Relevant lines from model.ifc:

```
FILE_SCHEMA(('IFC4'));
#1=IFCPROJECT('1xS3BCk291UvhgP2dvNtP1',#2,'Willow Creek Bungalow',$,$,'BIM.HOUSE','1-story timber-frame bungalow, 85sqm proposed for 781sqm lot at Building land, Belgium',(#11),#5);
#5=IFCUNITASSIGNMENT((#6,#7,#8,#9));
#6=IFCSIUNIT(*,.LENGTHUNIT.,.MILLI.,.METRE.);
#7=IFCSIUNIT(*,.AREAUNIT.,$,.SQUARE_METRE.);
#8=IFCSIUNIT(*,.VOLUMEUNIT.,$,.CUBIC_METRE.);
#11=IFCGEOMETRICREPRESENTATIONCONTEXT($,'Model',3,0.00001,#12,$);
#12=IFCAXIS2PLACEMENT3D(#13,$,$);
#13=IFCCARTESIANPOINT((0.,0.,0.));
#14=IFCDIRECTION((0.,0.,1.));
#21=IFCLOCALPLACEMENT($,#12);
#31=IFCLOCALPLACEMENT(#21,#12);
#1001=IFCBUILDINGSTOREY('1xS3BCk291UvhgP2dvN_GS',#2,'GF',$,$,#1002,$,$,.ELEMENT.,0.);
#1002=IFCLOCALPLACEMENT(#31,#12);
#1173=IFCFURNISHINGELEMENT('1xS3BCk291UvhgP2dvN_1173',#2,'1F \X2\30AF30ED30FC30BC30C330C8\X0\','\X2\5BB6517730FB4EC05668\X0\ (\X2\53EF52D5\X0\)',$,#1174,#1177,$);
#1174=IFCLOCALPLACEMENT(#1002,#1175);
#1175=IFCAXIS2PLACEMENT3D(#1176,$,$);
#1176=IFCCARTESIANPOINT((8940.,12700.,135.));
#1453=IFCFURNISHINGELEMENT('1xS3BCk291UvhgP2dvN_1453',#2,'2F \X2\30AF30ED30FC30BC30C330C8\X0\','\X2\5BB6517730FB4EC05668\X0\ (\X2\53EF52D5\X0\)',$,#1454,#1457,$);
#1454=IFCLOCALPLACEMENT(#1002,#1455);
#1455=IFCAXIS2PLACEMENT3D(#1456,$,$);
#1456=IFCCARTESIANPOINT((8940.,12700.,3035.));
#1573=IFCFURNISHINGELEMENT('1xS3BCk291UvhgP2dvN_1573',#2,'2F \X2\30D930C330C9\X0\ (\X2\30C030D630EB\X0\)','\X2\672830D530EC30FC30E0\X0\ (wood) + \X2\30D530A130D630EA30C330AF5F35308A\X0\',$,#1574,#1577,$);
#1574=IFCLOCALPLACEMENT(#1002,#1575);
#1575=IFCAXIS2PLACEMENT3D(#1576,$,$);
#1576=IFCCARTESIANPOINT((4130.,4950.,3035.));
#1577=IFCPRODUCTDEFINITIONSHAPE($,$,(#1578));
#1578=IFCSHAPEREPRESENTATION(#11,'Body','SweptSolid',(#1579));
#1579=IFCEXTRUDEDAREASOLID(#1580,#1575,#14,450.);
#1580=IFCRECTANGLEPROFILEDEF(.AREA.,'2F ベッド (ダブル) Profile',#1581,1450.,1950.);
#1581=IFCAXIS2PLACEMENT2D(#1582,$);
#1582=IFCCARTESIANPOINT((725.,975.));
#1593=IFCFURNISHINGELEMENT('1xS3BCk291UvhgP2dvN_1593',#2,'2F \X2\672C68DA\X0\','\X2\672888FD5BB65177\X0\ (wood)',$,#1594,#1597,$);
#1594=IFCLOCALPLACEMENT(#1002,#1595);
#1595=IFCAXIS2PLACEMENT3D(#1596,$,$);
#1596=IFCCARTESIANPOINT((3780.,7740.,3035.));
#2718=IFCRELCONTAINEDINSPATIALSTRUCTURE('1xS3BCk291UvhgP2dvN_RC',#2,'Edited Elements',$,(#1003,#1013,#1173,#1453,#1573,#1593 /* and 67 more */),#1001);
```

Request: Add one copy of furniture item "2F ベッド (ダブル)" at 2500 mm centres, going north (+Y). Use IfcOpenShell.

```python
import numpy as np
import ifcopenshell
import ifcopenshell.api.geometry
import ifcopenshell.api.root
import ifcopenshell.util.element
import ifcopenshell.util.placement

model = ifcopenshell.open("model.ifc")


def reuse_history(source, copy):
    """copy_class also copies each property set's owner history, people and application; keep the originals."""
    for rel in copy.IsDefinedBy:
        if rel.is_a("IfcRelDefinesByProperties") and (history := rel.RelatingPropertyDefinition.OwnerHistory):
            rel.RelatingPropertyDefinition.OwnerHistory = source.OwnerHistory
            ifcopenshell.util.element.remove_deep2(model, history)


source = model.by_id(1573)
base = ifcopenshell.util.placement.get_local_placement(source.ObjectPlacement)
step = np.array([0.0, 1.0, 0.0]) * 2500.0

for i in range(1, 2):
    copy = ifcopenshell.api.root.copy_class(model, product=source)
    copy.Representation = ifcopenshell.util.element.copy_deep(
        model, source.Representation, exclude=["IfcGeometricRepresentationContext", "IfcRepresentationMap"]
    )
    reuse_history(source, copy)
    matrix = base.copy()
    matrix[:3, 3] += i * step
    print("added at", matrix[:3, 3].round(3) + 0.0)
    ifcopenshell.api.geometry.edit_object_placement(model, product=copy, matrix=matrix, is_si=False)

model.write("model_v2.ifc")
```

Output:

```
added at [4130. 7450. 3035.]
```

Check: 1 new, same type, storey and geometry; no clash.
